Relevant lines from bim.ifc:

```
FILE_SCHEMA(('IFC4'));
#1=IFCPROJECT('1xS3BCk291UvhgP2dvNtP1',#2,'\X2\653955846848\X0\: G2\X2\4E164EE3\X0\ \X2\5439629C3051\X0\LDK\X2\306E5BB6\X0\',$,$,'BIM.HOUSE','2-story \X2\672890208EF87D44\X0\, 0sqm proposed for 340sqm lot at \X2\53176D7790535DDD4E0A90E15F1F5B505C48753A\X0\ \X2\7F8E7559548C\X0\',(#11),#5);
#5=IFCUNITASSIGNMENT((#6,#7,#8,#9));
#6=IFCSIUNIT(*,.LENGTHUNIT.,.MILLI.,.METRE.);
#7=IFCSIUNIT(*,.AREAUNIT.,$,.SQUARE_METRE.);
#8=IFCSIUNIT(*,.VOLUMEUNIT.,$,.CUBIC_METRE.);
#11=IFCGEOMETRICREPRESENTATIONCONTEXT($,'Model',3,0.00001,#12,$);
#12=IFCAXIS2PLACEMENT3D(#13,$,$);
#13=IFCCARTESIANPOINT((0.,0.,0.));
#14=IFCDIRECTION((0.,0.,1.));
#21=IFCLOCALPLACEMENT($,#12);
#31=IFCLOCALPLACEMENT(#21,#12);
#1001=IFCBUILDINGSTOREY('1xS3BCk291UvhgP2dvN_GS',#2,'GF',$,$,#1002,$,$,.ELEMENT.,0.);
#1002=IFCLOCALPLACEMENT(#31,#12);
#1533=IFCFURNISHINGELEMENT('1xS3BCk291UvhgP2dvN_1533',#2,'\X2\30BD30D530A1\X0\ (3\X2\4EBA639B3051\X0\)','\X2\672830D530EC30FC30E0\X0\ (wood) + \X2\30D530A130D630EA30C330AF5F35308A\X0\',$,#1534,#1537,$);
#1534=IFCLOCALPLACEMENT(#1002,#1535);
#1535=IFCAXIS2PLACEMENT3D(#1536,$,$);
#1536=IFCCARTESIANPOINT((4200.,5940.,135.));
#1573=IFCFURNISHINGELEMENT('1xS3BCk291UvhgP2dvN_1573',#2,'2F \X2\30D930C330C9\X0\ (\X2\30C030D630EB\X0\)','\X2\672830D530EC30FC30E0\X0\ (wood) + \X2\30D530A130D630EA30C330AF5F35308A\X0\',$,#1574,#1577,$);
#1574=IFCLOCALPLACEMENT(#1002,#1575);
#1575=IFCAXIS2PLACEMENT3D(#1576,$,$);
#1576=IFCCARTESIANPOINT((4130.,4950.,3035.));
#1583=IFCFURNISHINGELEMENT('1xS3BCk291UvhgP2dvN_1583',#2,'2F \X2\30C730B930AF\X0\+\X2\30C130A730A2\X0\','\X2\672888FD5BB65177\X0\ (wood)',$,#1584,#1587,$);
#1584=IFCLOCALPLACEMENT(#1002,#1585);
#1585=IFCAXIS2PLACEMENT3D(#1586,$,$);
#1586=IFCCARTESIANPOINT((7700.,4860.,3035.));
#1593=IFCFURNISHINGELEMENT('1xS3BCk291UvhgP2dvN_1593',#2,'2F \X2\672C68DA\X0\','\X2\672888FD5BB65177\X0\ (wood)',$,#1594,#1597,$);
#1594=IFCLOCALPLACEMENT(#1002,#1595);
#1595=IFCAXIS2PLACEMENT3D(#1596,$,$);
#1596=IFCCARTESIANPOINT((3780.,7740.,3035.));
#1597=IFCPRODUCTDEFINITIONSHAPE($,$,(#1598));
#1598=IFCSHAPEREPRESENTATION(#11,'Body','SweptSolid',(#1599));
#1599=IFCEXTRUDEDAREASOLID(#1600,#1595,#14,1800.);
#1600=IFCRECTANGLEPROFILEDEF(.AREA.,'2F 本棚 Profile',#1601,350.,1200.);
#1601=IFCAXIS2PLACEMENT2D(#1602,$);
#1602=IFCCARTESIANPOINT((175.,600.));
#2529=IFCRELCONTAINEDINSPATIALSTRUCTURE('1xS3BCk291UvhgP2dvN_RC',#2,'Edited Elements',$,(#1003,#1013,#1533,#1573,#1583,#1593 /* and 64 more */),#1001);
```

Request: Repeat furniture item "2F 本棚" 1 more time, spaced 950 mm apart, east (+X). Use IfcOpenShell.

```python
import numpy as np
import ifcopenshell
import ifcopenshell.api.geometry
import ifcopenshell.api.root
import ifcopenshell.util.element
import ifcopenshell.util.placement
import ifcopenshell.util.unit

model = ifcopenshell.open("bim.ifc")
unit_scale = ifcopenshell.util.unit.calculate_unit_scale(model)


def reuse_history(source, copy):
    """copy_class also copies each property set's owner history, people and application; keep the originals."""
    for rel in copy.IsDefinedBy:
        if rel.is_a("IfcRelDefinesByProperties") and (history := rel.RelatingPropertyDefinition.OwnerHistory):
            rel.RelatingPropertyDefinition.OwnerHistory = source.OwnerHistory
            ifcopenshell.util.element.remove_deep2(model, history)


source = model.by_guid("1xS3BCk291UvhgP2dvN_1593")
base = ifcopenshell.util.placement.get_local_placement(source.ObjectPlacement)
step = np.array([1.0, 0.0, 0.0]) * 0.95 / unit_scale

for i in range(1, 2):
    copy = ifcopenshell.api.root.copy_class(model, product=source)
    copy.Representation = ifcopenshell.util.element.copy_deep(
        model, source.Representation, exclude=["IfcGeometricRepresentationContext", "IfcRepresentationMap"]
    )
    reuse_history(source, copy)
    matrix = base.copy()
    matrix[:3, 3] += i * step
    print("added at", matrix[:3, 3].round(3) + 0.0)
    ifcopenshell.api.geometry.edit_object_placement(model, product=copy, matrix=matrix, is_si=False)

model.write("bim-out.ifc")
```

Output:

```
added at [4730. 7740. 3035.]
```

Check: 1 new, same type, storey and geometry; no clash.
